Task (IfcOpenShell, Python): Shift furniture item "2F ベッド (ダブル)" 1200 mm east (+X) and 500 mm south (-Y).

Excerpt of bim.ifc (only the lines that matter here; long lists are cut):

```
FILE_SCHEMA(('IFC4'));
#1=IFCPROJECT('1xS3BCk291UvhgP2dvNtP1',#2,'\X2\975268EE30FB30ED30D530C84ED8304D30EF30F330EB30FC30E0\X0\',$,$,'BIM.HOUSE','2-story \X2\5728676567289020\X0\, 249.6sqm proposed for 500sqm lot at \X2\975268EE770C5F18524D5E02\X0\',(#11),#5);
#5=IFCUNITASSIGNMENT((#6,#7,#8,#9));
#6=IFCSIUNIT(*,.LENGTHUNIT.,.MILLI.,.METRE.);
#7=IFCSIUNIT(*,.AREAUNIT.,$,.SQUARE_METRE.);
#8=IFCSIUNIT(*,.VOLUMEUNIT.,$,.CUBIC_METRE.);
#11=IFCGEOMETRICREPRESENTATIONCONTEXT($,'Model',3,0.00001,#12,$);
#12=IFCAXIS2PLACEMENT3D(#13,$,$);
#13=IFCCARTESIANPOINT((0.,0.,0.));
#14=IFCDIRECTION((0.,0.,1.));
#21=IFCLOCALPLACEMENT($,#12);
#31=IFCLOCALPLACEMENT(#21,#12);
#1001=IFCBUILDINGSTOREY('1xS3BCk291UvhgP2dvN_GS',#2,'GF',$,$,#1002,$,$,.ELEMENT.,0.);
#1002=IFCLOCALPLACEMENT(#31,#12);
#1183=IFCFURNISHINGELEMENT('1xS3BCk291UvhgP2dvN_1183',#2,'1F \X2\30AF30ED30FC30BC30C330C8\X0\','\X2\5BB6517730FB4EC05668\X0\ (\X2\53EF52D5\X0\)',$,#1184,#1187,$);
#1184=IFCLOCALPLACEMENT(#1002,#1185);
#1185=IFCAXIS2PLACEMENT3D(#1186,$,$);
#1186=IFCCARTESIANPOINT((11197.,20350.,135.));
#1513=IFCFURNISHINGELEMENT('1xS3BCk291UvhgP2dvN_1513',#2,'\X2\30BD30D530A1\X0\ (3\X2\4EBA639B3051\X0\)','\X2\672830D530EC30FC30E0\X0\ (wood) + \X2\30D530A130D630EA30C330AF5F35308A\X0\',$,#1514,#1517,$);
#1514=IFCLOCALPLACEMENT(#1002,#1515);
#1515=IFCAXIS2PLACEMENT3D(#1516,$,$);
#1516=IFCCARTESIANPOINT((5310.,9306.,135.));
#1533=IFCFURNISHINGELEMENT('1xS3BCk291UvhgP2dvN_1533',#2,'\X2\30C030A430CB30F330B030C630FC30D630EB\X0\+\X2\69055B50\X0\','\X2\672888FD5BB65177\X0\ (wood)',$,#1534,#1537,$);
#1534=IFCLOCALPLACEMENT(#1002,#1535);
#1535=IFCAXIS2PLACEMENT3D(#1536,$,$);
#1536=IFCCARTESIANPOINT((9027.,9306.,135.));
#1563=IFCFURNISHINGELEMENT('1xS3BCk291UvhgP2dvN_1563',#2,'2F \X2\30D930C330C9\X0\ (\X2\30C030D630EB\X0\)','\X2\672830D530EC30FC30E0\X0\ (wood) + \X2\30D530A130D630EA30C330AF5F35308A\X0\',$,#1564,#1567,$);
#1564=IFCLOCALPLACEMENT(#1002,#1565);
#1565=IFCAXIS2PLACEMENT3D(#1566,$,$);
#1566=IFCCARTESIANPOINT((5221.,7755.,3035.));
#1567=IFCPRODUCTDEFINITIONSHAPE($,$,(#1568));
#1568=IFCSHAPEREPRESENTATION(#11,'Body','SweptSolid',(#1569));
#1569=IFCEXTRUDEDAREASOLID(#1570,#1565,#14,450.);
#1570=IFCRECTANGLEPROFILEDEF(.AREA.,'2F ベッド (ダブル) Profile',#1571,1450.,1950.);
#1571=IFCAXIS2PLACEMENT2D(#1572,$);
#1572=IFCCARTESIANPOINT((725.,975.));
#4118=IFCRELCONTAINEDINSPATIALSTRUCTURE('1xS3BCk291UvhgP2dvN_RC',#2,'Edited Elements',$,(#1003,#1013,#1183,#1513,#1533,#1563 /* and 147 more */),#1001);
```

```python
import ifcopenshell
import ifcopenshell.api.geometry
import ifcopenshell.util.placement
import ifcopenshell.util.unit

model = ifcopenshell.open("bim.ifc")
unit_scale = ifcopenshell.util.unit.calculate_unit_scale(model)

item = model.by_guid("1xS3BCk291UvhgP2dvN_1563")
matrix = ifcopenshell.util.placement.get_local_placement(item.ObjectPlacement)
matrix[0, 3] += 1.2 / unit_scale
matrix[1, 3] -= 0.5 / unit_scale
ifcopenshell.api.geometry.edit_object_placement(model, product=item, matrix=matrix, is_si=False)

print(ifcopenshell.util.placement.get_local_placement(item.ObjectPlacement).round(3) + 0.0)

model.write("bim_rev.ifc")
```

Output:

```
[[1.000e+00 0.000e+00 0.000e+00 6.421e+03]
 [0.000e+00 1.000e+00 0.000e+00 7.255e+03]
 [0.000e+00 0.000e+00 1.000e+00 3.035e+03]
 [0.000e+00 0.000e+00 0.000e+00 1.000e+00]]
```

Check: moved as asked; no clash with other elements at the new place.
